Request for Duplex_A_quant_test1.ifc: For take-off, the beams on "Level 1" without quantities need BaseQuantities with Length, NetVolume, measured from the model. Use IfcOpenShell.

First a look at what the model holds.

```python
import ifcopenshell
import ifcopenshell.util.element
import ifcopenshell.util.unit

model = ifcopenshell.open("Duplex_A_quant_test1.ifc")
print(model.schema)
for unit_type in ("LENGTHUNIT", "AREAUNIT", "VOLUMEUNIT"):
    print(unit_type, ifcopenshell.util.unit.calculate_unit_scale(model, unit_type))
storey = next(s for s in model.by_type("IfcBuildingStorey") if s.Name == "Level 1")
beams = [e for e in ifcopenshell.util.element.get_decomposition(storey) if e.is_a("IfcBeam")]
for e in sorted(beams, key=lambda e: e.id()):
    print(e.id(), e.is_a(), e.Name, list(ifcopenshell.util.element.get_psets(e, qtos_only=True)), sep=" | ")
```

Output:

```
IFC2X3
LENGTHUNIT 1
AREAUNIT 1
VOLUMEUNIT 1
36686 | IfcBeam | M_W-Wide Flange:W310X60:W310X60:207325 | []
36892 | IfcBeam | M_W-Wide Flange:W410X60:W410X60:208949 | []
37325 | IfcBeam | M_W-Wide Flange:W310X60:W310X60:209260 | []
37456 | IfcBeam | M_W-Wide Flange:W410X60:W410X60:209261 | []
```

```python
import ifcopenshell
import ifcopenshell.api.pset
import ifcopenshell.geom
import ifcopenshell.util.element
import ifcopenshell.util.shape
import ifcopenshell.util.unit

model = ifcopenshell.open("Duplex_A_quant_test1.ifc")
unit_scale = ifcopenshell.util.unit.calculate_unit_scale(model)
volume_scale = ifcopenshell.util.unit.calculate_unit_scale(model, "VOLUMEUNIT")
settings = ifcopenshell.geom.settings()

storey = next(s for s in model.by_type("IfcBuildingStorey") if s.Name == "Level 1")
beams = [e for e in ifcopenshell.util.element.get_decomposition(storey) if e.is_a("IfcBeam")]

for e in sorted(beams, key=lambda e: e.id()):
    if ifcopenshell.util.element.get_psets(e, qtos_only=True, should_inherit=False):
        continue
    # Geometry comes back in metres, in the element's own axes.
    shape = ifcopenshell.geom.create_shape(settings, e)
    values = {
        "Length": ifcopenshell.util.shape.get_max_xyz(shape.geometry) / unit_scale,
        "NetVolume": ifcopenshell.util.shape.get_volume(shape.geometry) / volume_scale,
    }
    qto = ifcopenshell.api.pset.add_qto(model, product=e, name="BaseQuantities")
    ifcopenshell.api.pset.edit_qto(model, qto=qto, properties=values)
    print(e.id(), {k: round(v, 3) for k, v in values.items()})

model.write("Duplex_A_quant_test1_v2.ifc")
```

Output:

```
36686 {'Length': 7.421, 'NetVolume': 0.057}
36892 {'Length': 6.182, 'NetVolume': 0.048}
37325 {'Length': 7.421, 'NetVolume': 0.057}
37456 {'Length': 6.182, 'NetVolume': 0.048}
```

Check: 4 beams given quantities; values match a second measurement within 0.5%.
